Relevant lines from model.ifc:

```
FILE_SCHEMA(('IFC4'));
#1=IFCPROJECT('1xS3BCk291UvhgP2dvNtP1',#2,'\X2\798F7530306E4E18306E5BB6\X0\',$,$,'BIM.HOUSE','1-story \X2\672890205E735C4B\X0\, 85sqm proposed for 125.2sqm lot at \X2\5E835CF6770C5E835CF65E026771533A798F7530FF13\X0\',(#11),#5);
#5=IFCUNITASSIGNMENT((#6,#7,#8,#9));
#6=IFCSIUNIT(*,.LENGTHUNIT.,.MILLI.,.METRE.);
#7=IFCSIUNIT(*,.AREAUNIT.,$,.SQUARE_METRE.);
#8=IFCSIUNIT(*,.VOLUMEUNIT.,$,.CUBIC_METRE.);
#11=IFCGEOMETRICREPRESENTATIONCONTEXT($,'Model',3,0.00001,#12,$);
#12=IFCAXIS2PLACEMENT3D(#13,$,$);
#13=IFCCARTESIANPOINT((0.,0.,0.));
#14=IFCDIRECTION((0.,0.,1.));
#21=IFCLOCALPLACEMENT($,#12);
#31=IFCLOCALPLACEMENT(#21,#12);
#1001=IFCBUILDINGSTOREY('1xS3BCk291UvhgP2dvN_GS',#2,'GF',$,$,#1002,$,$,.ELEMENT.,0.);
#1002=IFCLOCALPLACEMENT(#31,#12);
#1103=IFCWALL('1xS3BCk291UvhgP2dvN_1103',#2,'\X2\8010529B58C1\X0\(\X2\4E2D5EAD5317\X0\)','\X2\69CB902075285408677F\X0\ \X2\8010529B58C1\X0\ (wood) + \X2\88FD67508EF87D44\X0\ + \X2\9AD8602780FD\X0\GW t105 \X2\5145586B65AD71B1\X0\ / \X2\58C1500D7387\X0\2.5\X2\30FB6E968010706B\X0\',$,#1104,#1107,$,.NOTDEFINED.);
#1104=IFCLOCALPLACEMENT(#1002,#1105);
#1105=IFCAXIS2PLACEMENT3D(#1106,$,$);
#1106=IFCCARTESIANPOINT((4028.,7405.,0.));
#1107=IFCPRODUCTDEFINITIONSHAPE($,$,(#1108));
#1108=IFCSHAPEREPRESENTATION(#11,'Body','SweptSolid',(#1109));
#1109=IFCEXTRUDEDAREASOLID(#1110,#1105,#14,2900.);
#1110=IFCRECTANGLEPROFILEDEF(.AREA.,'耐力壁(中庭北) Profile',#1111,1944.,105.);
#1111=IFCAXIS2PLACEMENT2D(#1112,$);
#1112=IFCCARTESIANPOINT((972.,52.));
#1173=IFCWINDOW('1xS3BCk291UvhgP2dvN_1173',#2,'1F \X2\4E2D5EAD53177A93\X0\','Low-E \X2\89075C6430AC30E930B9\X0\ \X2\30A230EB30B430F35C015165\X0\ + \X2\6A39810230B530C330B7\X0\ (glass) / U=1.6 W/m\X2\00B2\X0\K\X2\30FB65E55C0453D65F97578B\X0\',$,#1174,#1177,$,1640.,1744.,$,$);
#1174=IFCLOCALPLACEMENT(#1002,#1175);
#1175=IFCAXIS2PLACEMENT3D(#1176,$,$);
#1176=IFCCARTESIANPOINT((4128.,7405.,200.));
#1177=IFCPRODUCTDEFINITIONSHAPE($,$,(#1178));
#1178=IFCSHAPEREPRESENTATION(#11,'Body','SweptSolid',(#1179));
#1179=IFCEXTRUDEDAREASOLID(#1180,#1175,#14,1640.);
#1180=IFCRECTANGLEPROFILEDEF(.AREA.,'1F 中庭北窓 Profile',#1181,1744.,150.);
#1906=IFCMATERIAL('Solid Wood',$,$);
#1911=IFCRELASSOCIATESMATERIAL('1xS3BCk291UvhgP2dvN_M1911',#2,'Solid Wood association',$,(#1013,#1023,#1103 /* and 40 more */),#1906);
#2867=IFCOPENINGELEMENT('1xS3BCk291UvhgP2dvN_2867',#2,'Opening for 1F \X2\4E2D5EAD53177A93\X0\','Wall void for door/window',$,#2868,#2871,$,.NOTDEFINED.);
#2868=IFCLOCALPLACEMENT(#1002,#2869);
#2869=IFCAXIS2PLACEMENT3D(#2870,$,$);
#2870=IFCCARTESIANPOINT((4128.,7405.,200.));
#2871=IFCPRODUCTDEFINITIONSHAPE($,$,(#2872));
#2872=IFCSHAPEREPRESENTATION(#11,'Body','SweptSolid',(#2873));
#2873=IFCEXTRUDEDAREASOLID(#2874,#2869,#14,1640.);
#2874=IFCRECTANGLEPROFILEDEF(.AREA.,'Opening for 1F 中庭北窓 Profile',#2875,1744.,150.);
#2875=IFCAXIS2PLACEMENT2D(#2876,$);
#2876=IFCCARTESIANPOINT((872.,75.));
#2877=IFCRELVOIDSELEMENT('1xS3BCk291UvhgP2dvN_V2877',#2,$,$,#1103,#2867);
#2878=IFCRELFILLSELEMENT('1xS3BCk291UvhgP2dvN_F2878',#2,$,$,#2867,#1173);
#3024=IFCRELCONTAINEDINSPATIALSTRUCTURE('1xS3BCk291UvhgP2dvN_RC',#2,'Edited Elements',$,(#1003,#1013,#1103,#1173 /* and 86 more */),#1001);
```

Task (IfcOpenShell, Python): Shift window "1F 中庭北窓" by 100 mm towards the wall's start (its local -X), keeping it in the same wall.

```python
import ifcopenshell
import ifcopenshell.api.geometry
import ifcopenshell.util.placement
import ifcopenshell.util.unit

model = ifcopenshell.open("model.ifc")
unit_scale = ifcopenshell.util.unit.calculate_unit_scale(model)

window = model.by_guid("1xS3BCk291UvhgP2dvN_1173")
opening = window.FillsVoids[0].RelatingOpeningElement
wall = opening.VoidsElements[0].RelatingBuildingElement

wall_matrix = ifcopenshell.util.placement.get_local_placement(wall.ObjectPlacement)
shift = wall_matrix[:3, 0] * -0.1 / unit_scale
before = ifcopenshell.util.placement.get_local_placement(window.ObjectPlacement)[:3, 3].copy()

# The window is not placed relative to its opening, so move both.
for product in (opening, window):
    matrix = ifcopenshell.util.placement.get_local_placement(product.ObjectPlacement)
    matrix[:3, 3] += shift
    ifcopenshell.api.geometry.edit_object_placement(model, product=product, matrix=matrix, is_si=False)

after = ifcopenshell.util.placement.get_local_placement(window.ObjectPlacement)[:3, 3]
print("window moved by", (after - before).round(3) + 0.0)

model.write("model_edited.ifc")
```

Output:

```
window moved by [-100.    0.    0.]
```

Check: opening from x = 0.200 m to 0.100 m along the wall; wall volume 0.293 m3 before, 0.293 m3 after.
